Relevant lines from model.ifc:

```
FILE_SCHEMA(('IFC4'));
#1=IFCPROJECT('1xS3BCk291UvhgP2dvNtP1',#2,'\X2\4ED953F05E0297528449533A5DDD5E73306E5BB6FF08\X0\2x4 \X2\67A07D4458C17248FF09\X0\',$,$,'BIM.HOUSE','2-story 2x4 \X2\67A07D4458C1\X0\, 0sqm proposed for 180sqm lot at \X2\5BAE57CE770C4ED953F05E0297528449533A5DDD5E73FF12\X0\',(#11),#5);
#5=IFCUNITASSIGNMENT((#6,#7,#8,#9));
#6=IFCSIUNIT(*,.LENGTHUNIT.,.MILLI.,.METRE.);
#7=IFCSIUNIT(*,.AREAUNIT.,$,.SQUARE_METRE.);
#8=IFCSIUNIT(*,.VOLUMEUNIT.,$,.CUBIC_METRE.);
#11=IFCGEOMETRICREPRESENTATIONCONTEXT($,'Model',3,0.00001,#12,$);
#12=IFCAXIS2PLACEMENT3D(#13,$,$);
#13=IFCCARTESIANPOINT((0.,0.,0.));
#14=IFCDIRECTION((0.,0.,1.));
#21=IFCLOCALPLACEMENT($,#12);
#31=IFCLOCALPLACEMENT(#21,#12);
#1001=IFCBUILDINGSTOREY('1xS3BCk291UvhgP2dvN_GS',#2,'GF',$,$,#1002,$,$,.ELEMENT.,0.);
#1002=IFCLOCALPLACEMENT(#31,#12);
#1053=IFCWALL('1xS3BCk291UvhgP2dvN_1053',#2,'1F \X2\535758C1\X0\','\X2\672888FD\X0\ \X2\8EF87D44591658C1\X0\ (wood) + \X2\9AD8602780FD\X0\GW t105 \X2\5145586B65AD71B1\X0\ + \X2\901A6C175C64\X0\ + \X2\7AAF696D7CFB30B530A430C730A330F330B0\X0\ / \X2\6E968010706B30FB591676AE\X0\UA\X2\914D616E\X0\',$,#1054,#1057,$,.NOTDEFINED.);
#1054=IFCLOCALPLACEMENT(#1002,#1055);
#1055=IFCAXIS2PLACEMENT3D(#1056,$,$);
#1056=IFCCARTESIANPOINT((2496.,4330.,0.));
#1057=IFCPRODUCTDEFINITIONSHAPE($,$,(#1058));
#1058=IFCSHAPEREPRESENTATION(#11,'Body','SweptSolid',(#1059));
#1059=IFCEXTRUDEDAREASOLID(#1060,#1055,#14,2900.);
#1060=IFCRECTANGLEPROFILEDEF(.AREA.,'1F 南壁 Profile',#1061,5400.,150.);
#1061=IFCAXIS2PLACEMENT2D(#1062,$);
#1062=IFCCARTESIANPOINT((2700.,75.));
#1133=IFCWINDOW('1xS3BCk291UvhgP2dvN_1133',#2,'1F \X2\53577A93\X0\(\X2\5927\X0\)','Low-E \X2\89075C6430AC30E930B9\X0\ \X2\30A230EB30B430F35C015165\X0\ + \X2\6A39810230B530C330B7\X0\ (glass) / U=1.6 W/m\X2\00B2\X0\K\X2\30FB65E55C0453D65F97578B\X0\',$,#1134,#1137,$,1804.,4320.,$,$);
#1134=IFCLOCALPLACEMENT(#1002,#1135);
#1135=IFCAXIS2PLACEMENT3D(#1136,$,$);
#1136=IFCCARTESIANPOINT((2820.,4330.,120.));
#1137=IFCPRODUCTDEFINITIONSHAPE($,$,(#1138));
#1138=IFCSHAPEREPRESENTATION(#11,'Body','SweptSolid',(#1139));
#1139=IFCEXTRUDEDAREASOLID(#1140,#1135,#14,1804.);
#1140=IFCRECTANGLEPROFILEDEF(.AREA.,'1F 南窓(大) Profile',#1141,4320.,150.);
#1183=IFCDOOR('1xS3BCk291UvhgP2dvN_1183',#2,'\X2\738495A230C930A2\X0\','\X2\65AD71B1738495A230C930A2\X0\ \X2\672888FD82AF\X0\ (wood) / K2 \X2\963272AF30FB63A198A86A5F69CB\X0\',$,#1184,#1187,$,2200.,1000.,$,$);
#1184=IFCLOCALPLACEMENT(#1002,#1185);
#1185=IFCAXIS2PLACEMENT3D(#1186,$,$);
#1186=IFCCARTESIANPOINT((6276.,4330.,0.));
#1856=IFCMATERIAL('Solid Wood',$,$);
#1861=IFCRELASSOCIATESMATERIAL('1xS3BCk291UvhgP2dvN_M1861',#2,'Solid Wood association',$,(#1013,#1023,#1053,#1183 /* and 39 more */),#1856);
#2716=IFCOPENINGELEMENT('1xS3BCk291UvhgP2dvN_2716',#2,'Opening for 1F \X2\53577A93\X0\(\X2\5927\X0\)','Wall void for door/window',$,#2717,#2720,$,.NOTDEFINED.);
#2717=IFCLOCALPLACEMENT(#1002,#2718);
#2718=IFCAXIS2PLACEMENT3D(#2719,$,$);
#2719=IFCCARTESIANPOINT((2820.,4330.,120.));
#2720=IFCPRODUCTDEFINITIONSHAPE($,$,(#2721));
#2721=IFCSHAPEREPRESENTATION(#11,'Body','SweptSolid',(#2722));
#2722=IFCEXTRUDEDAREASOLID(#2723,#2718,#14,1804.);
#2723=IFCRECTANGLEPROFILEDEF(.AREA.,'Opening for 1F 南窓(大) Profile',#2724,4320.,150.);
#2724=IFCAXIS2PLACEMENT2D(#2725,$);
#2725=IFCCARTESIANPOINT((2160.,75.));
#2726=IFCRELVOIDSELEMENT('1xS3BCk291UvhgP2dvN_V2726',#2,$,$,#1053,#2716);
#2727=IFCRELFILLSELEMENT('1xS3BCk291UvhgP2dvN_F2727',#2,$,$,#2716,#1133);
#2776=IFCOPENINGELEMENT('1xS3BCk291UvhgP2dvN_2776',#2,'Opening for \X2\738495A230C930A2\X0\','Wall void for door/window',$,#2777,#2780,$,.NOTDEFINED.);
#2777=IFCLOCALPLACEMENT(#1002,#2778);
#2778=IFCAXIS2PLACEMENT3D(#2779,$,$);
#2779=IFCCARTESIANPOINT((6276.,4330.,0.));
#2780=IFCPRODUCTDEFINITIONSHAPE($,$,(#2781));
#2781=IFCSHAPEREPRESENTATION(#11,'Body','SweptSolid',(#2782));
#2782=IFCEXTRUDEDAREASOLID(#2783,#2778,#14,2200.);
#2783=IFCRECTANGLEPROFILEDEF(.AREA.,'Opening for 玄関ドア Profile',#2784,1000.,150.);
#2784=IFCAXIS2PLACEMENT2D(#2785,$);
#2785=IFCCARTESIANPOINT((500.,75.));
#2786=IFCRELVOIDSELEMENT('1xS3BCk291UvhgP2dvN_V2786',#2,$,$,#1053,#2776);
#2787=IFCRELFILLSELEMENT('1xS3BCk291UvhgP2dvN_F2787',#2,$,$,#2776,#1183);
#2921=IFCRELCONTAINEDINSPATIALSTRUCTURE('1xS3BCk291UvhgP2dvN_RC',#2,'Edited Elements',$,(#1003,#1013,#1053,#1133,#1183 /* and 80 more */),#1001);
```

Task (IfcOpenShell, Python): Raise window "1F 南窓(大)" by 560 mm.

```python
import numpy as np
import ifcopenshell
import ifcopenshell.api.geometry
import ifcopenshell.util.placement
import ifcopenshell.util.unit

model = ifcopenshell.open("model.ifc")
unit_scale = ifcopenshell.util.unit.calculate_unit_scale(model)

window = model.by_guid("1xS3BCk291UvhgP2dvN_1133")
opening = window.FillsVoids[0].RelatingOpeningElement
dz = 560.0

shift = np.array([0.0, 0.0, dz])
# The window is not placed relative to its opening, so move both.
for product in (opening, window):
    matrix = ifcopenshell.util.placement.get_local_placement(product.ObjectPlacement)
    matrix[:3, 3] += shift
    ifcopenshell.api.geometry.edit_object_placement(model, product=product, matrix=matrix, is_si=False)

print(f"moved by {dz * unit_scale:+.3f} m")

model.write("model_v2.ifc")
```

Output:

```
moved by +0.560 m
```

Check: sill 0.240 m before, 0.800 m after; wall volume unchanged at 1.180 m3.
